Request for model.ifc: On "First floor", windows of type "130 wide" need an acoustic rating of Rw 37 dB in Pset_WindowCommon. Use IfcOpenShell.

First a look at what the model holds.

```python
import ifcopenshell
import ifcopenshell.util.element

model = ifcopenshell.open("model.ifc")
print(model.schema)
storey = next(s for s in model.by_type("IfcBuildingStorey") if s.Name == "First floor")
windows = [e for e in ifcopenshell.util.element.get_decomposition(storey) if e.is_a("IfcWindow")]
seen = {}
for e in windows:
    element_type = ifcopenshell.util.element.get_type(e)
    key = (element_type.Name if element_type != e and element_type else None, ifcopenshell.util.element.get_pset(e, "Pset_WindowCommon", "AcousticRating"))
    seen[key] = seen.get(key, 0) + 1
for (name, value), count in sorted(seen.items(), key=str):
    print(count, "x", name, "|", value)
```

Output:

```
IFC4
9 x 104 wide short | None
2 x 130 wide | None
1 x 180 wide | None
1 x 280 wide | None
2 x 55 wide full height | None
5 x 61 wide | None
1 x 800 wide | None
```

```python
import ifcopenshell
import ifcopenshell.api.pset
import ifcopenshell.util.element

model = ifcopenshell.open("model.ifc")

storey = next(s for s in model.by_type("IfcBuildingStorey") if s.Name == "First floor")
windows = [e for e in ifcopenshell.util.element.get_decomposition(storey) if e.is_a("IfcWindow")]

count = 0
for e in windows:
    element_type = ifcopenshell.util.element.get_type(e)
    if element_type in (None, e) or element_type.Name != "130 wide":
        continue
    # add_pset returns the element's existing set when there is one.
    pset = ifcopenshell.api.pset.add_pset(model, product=e, name="Pset_WindowCommon")
    ifcopenshell.api.pset.edit_pset(model, pset=pset, properties={"AcousticRating": "Rw 37 dB"})
    count += 1

print(count, "windows updated")

model.write("model_edited.ifc")
```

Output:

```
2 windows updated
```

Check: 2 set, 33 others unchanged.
